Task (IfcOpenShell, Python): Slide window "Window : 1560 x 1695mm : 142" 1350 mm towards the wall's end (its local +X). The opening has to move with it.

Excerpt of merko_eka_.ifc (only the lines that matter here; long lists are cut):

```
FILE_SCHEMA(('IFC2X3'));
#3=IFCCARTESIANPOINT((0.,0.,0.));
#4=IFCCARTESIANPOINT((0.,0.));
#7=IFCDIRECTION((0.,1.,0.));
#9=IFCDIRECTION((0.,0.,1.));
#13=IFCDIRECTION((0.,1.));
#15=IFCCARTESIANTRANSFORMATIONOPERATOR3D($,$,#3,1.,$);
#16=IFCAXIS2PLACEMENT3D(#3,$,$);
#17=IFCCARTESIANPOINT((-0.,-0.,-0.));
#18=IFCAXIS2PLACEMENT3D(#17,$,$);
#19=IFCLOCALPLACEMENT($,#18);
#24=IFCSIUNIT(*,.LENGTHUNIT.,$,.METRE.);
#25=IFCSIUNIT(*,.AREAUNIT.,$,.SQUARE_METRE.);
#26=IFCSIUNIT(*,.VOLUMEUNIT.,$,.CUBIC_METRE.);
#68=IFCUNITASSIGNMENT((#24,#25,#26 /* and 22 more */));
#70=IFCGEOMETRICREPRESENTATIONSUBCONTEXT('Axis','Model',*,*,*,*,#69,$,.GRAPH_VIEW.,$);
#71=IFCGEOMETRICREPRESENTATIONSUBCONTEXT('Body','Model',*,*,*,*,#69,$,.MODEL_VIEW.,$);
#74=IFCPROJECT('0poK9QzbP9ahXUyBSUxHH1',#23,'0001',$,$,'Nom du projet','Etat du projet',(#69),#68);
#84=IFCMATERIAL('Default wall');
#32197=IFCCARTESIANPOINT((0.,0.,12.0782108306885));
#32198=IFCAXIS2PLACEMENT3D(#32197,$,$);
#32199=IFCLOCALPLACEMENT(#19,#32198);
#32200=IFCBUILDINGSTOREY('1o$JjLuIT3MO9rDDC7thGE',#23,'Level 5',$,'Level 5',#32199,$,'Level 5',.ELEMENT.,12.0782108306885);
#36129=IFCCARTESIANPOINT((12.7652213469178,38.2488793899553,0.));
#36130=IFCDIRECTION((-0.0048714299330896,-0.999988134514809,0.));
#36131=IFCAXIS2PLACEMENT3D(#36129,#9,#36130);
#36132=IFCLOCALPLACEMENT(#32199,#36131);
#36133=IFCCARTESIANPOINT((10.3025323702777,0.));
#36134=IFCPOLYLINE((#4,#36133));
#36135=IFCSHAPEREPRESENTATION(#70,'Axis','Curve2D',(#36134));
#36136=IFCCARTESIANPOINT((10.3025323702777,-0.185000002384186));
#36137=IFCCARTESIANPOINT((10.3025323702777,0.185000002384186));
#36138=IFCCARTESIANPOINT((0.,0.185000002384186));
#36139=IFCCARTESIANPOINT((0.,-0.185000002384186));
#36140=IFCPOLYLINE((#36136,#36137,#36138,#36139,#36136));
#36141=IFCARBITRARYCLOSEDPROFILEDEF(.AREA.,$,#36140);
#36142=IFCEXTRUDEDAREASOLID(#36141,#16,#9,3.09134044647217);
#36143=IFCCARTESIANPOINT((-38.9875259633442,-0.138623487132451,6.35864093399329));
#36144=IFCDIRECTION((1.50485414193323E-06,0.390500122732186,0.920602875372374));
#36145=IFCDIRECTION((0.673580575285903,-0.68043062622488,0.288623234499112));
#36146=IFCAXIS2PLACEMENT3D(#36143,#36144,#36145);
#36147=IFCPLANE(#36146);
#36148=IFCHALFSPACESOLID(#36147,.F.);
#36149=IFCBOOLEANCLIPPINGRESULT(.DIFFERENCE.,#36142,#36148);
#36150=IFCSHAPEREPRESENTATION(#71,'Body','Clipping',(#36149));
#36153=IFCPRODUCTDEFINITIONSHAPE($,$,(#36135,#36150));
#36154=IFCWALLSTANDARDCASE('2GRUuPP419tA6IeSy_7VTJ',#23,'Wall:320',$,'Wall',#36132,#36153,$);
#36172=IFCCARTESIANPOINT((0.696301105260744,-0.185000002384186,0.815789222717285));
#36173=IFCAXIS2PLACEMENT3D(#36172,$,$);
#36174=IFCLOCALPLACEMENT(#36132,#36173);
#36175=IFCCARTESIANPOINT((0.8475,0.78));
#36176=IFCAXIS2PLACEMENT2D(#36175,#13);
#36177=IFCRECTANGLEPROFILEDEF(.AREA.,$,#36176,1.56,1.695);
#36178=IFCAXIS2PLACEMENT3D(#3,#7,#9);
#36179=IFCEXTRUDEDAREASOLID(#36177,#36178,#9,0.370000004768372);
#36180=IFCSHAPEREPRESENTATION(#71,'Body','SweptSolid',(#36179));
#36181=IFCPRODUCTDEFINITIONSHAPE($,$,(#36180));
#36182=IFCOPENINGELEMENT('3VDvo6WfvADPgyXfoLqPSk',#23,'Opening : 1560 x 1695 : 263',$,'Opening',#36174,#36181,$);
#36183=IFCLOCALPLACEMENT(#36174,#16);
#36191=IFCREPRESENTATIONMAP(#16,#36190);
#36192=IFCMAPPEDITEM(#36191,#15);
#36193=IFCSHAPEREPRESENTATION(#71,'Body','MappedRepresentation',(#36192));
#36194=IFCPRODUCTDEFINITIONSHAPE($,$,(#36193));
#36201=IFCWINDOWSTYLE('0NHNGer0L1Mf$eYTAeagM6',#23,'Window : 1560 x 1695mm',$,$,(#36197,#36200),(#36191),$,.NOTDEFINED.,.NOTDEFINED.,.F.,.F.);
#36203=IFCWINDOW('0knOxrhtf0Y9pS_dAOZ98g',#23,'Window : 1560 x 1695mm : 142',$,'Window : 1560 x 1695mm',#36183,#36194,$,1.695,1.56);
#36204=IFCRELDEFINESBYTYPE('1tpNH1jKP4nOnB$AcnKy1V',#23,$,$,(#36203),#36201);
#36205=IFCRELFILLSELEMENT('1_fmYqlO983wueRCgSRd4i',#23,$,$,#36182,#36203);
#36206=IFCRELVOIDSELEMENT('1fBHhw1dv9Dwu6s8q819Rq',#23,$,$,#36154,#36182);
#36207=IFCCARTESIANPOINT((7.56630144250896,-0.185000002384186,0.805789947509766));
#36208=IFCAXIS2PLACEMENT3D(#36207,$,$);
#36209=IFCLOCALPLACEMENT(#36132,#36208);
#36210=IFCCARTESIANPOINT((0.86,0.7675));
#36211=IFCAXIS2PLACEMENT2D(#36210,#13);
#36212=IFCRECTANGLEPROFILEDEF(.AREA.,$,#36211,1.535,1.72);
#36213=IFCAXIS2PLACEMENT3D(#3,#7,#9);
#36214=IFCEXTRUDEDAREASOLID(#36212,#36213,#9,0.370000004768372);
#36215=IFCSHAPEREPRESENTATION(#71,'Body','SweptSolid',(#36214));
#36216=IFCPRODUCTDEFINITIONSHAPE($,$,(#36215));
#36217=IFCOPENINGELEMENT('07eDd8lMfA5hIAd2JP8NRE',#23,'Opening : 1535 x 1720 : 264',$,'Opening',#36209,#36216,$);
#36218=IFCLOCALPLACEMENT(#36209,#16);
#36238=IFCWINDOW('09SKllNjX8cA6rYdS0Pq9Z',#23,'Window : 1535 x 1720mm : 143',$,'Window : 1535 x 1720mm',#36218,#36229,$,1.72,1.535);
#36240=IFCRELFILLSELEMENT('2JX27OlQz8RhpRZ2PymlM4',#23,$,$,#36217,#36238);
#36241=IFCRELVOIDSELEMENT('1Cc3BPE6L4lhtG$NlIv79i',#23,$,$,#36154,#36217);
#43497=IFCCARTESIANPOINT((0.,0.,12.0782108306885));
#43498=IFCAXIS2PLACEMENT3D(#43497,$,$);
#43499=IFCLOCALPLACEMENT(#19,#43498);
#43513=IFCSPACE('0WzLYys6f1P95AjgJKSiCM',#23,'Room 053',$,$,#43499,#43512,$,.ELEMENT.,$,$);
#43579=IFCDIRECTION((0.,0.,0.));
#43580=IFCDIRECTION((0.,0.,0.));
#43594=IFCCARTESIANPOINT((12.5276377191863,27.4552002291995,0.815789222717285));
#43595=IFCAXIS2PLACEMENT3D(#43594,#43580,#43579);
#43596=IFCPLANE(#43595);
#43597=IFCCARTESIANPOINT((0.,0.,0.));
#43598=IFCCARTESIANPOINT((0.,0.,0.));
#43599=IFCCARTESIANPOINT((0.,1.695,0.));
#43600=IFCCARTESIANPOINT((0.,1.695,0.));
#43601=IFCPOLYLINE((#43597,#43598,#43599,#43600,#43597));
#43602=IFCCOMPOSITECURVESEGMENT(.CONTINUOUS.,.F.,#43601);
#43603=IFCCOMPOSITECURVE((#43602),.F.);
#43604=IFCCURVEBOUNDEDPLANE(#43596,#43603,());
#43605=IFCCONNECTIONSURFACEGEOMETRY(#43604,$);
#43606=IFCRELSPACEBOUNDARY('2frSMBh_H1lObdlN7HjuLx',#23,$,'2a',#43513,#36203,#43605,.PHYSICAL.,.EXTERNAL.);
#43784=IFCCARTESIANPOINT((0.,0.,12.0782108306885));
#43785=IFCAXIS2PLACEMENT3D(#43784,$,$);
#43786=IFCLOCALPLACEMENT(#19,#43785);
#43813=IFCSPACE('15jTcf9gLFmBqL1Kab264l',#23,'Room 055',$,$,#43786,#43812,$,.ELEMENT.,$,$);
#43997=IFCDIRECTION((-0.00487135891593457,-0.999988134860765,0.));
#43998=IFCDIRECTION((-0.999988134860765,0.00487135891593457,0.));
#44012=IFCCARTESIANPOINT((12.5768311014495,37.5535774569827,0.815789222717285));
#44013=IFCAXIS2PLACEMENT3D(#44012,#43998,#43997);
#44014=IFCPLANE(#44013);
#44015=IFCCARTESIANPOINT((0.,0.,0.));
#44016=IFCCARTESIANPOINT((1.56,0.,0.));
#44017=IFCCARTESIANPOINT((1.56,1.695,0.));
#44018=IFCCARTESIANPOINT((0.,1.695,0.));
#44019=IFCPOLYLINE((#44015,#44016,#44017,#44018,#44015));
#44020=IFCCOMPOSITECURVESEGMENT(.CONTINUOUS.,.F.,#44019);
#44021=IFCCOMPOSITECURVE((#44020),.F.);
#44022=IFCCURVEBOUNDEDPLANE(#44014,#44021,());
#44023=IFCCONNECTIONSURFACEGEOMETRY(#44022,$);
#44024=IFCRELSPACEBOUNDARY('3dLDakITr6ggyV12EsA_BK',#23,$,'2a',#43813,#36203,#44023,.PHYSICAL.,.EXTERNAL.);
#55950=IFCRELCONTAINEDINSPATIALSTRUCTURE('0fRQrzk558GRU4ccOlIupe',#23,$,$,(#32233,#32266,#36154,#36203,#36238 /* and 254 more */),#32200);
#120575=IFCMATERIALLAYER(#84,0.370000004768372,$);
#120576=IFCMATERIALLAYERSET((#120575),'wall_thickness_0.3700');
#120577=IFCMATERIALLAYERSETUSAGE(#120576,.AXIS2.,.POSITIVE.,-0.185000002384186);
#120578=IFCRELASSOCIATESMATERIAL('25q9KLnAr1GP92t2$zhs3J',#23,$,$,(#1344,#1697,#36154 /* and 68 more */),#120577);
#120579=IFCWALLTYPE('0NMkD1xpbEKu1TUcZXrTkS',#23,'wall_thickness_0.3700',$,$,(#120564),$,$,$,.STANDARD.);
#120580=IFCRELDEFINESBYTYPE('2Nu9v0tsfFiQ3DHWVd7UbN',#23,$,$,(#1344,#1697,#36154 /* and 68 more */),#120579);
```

```python
import numpy as np
import ifcopenshell
import ifcopenshell.api.geometry
import ifcopenshell.util.placement
import ifcopenshell.util.unit

model = ifcopenshell.open("merko_eka_.ifc")
unit_scale = ifcopenshell.util.unit.calculate_unit_scale(model)

window = model.by_guid("0knOxrhtf0Y9pS_dAOZ98g")
opening = window.FillsVoids[0].RelatingOpeningElement
wall = opening.VoidsElements[0].RelatingBuildingElement

wall_matrix = ifcopenshell.util.placement.get_local_placement(wall.ObjectPlacement)
shift = wall_matrix[:3, 0] * 1.35 / unit_scale
before = ifcopenshell.util.placement.get_local_placement(window.ObjectPlacement)[:3, 3].copy()

# The window is placed relative to its opening, so it follows when the opening moves.
matrix = ifcopenshell.util.placement.get_local_placement(opening.ObjectPlacement)
matrix[:3, 3] += shift
ifcopenshell.api.geometry.edit_object_placement(
    model, product=opening, matrix=matrix, is_si=False, should_transform_children=True
)

# Space boundary surfaces are stored in each space's coordinates; move them too.
for rel in window.ProvidesBoundaries:
    if not rel.ConnectionGeometry:
        continue
    surface = rel.ConnectionGeometry.SurfaceOnRelatingElement.BasisSurface
    space_matrix = ifcopenshell.util.placement.get_local_placement(rel.RelatingSpace.ObjectPlacement)
    point = np.array(surface.Position.Location.Coordinates) + space_matrix[:3, :3].T @ shift
    surface.Position = model.createIfcAxis2Placement3D(
        model.createIfcCartesianPoint(point.tolist()), surface.Position.Axis, surface.Position.RefDirection
    )

after = ifcopenshell.util.placement.get_local_placement(window.ObjectPlacement)[:3, 3]
print("window moved by", (after - before).round(3) + 0.0)

model.write("merko_eka__updated.ifc")
```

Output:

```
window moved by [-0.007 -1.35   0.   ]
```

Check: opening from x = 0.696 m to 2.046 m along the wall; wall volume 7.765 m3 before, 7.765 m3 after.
